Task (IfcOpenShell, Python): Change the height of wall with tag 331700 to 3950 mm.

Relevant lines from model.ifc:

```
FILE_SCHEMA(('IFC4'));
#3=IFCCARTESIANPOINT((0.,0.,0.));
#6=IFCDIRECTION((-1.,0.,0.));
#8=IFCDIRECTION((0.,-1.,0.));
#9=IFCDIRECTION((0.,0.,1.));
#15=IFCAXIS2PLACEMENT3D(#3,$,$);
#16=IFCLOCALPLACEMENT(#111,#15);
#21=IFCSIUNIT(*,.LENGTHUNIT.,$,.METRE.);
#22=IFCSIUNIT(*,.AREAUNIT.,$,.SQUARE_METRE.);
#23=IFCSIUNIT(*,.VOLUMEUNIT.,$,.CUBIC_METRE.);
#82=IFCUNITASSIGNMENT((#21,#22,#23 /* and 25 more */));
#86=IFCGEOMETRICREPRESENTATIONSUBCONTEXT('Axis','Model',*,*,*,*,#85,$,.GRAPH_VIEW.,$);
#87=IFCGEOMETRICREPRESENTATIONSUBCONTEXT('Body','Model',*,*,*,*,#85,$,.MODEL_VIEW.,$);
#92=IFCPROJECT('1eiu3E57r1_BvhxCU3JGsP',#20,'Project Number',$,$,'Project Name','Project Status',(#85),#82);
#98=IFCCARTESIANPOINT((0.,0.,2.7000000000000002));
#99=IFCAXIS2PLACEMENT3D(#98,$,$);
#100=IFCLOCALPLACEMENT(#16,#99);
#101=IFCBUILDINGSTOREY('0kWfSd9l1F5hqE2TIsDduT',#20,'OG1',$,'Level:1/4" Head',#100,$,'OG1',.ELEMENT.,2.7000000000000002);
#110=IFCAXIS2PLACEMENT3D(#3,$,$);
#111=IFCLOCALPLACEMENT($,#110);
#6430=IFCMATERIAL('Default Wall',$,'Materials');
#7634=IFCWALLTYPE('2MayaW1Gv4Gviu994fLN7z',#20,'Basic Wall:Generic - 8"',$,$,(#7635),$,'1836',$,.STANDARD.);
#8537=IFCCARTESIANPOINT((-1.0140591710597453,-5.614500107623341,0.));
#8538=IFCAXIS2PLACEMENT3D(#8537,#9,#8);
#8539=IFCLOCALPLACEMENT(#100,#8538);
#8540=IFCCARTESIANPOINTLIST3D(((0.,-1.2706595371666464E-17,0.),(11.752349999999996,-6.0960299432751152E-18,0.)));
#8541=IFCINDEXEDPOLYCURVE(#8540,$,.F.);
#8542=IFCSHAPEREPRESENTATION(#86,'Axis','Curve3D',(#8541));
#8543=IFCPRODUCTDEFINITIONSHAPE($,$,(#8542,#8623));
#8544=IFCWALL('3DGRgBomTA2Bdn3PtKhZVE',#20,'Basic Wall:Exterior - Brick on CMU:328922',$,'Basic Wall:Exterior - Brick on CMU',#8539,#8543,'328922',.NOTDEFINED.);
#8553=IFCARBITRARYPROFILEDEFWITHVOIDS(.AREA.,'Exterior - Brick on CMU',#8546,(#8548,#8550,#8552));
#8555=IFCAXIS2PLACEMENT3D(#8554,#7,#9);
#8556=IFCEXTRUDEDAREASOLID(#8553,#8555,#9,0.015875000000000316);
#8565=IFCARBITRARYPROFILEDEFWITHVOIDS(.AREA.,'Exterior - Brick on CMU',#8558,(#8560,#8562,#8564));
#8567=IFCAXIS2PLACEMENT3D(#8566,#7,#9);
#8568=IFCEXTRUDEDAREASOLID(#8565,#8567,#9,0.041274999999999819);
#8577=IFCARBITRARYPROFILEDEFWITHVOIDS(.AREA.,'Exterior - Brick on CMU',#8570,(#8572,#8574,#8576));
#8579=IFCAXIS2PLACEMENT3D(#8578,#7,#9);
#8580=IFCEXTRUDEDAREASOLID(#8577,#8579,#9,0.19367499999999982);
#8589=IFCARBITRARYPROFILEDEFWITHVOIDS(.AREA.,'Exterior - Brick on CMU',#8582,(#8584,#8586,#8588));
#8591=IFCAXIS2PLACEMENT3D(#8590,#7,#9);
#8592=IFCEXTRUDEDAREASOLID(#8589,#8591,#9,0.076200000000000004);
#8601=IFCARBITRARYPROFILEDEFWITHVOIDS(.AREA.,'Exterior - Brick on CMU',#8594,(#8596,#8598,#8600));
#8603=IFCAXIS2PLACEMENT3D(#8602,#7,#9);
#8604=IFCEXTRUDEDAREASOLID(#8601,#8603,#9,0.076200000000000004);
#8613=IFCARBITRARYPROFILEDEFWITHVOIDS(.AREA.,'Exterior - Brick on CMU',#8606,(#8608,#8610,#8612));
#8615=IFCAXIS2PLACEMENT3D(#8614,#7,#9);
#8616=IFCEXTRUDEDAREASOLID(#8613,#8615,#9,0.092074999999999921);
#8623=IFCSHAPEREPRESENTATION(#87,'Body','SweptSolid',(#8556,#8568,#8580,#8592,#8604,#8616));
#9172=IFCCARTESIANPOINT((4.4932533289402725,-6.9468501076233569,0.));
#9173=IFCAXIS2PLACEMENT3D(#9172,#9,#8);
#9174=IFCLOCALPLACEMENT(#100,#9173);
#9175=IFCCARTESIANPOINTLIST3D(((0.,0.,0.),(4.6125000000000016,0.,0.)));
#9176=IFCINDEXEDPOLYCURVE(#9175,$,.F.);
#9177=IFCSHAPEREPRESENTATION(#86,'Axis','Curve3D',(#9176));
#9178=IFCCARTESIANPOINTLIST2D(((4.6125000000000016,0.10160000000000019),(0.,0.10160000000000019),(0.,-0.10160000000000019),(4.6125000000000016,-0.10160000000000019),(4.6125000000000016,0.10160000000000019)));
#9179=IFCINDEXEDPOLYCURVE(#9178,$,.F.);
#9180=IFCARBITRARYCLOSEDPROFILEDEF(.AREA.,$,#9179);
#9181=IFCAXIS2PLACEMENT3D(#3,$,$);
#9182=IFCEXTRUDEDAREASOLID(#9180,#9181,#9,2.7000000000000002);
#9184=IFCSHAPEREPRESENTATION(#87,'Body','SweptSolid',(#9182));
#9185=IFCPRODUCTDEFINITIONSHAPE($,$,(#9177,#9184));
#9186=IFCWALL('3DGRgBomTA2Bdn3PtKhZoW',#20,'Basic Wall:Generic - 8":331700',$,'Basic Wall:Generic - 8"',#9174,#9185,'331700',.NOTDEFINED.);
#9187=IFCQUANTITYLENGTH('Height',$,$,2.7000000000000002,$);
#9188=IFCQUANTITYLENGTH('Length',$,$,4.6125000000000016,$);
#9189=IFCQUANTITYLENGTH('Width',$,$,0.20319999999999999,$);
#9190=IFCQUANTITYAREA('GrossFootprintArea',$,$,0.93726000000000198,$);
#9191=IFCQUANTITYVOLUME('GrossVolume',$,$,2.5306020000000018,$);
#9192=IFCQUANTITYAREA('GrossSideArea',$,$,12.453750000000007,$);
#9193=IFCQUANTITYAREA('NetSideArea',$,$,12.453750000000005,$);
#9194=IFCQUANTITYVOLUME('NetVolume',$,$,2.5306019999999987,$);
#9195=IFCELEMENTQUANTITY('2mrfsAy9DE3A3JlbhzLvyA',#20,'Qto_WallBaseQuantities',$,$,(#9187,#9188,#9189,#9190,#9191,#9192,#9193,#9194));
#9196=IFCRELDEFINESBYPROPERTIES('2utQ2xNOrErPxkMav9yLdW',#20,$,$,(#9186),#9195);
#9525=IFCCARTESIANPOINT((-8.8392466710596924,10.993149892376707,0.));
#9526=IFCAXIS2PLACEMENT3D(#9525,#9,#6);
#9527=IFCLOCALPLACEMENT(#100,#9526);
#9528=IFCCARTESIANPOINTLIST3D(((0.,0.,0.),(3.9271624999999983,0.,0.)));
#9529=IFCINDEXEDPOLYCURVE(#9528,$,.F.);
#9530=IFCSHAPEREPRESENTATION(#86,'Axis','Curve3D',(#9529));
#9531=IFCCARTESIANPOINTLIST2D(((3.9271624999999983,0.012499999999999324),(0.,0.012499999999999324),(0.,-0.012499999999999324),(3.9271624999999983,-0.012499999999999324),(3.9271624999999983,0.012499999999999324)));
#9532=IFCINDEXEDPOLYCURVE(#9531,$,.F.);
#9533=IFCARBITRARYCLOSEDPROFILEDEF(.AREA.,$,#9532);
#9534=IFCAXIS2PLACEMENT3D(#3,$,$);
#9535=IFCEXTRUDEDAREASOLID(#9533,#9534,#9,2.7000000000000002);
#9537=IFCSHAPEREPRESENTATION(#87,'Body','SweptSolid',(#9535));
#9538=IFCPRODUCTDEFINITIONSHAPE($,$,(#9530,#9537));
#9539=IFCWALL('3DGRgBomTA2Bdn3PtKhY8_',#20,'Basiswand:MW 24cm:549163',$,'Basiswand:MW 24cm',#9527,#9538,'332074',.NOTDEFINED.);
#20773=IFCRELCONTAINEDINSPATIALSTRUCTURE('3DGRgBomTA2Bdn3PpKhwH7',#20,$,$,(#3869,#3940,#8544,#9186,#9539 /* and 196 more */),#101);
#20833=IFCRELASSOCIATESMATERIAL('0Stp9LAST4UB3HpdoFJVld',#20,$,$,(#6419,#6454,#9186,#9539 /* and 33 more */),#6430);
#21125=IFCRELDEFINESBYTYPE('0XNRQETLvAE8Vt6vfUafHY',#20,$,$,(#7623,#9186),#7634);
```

```python
import ifcopenshell
import ifcopenshell.api.pset
import ifcopenshell.geom
import ifcopenshell.util.element
import ifcopenshell.util.representation
import ifcopenshell.util.shape
import ifcopenshell.util.unit

model = ifcopenshell.open("model.ifc")
unit_scale = ifcopenshell.util.unit.calculate_unit_scale(model)
area_scale = ifcopenshell.util.unit.calculate_unit_scale(model, "AREAUNIT")
volume_scale = ifcopenshell.util.unit.calculate_unit_scale(model, "VOLUMEUNIT")
settings = ifcopenshell.geom.settings()


def volume(element):
    """Net volume in cubic metres, openings subtracted."""
    shape = ifcopenshell.geom.create_shape(settings, element)
    return ifcopenshell.util.shape.get_volume(shape.geometry)


wall = model.by_id(9186)
before = volume(wall)

body = ifcopenshell.util.representation.get_representation(wall, "Model", "Body")
solid = body.Items[0]
old_height = solid.Depth
solid.Depth = 3.95 / unit_scale
after = volume(wall)
thickness = 0.2032  # wall thickness in metres

# Update the stored height, areas and volumes.
qto = model.by_id(ifcopenshell.util.element.get_pset(wall, "Qto_WallBaseQuantities", should_inherit=False)["id"])
ifcopenshell.api.pset.edit_qto(model, qto=qto, properties={
    "Height": solid.Depth,
    "GrossVolume": ifcopenshell.util.element.get_pset(wall, "Qto_WallBaseQuantities", "GrossVolume") * solid.Depth / old_height,
    "GrossSideArea": ifcopenshell.util.element.get_pset(wall, "Qto_WallBaseQuantities", "GrossSideArea") * solid.Depth / old_height,
    "NetSideArea": after / thickness / area_scale,
    "NetVolume": after / volume_scale,
})

print(f"height {old_height:g} -> {solid.Depth:g}, volume {before:.3f} -> {after:.3f} m3")

model.write("model_rev.ifc")
```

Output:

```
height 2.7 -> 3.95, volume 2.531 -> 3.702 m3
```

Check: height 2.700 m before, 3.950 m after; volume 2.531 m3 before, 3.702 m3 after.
